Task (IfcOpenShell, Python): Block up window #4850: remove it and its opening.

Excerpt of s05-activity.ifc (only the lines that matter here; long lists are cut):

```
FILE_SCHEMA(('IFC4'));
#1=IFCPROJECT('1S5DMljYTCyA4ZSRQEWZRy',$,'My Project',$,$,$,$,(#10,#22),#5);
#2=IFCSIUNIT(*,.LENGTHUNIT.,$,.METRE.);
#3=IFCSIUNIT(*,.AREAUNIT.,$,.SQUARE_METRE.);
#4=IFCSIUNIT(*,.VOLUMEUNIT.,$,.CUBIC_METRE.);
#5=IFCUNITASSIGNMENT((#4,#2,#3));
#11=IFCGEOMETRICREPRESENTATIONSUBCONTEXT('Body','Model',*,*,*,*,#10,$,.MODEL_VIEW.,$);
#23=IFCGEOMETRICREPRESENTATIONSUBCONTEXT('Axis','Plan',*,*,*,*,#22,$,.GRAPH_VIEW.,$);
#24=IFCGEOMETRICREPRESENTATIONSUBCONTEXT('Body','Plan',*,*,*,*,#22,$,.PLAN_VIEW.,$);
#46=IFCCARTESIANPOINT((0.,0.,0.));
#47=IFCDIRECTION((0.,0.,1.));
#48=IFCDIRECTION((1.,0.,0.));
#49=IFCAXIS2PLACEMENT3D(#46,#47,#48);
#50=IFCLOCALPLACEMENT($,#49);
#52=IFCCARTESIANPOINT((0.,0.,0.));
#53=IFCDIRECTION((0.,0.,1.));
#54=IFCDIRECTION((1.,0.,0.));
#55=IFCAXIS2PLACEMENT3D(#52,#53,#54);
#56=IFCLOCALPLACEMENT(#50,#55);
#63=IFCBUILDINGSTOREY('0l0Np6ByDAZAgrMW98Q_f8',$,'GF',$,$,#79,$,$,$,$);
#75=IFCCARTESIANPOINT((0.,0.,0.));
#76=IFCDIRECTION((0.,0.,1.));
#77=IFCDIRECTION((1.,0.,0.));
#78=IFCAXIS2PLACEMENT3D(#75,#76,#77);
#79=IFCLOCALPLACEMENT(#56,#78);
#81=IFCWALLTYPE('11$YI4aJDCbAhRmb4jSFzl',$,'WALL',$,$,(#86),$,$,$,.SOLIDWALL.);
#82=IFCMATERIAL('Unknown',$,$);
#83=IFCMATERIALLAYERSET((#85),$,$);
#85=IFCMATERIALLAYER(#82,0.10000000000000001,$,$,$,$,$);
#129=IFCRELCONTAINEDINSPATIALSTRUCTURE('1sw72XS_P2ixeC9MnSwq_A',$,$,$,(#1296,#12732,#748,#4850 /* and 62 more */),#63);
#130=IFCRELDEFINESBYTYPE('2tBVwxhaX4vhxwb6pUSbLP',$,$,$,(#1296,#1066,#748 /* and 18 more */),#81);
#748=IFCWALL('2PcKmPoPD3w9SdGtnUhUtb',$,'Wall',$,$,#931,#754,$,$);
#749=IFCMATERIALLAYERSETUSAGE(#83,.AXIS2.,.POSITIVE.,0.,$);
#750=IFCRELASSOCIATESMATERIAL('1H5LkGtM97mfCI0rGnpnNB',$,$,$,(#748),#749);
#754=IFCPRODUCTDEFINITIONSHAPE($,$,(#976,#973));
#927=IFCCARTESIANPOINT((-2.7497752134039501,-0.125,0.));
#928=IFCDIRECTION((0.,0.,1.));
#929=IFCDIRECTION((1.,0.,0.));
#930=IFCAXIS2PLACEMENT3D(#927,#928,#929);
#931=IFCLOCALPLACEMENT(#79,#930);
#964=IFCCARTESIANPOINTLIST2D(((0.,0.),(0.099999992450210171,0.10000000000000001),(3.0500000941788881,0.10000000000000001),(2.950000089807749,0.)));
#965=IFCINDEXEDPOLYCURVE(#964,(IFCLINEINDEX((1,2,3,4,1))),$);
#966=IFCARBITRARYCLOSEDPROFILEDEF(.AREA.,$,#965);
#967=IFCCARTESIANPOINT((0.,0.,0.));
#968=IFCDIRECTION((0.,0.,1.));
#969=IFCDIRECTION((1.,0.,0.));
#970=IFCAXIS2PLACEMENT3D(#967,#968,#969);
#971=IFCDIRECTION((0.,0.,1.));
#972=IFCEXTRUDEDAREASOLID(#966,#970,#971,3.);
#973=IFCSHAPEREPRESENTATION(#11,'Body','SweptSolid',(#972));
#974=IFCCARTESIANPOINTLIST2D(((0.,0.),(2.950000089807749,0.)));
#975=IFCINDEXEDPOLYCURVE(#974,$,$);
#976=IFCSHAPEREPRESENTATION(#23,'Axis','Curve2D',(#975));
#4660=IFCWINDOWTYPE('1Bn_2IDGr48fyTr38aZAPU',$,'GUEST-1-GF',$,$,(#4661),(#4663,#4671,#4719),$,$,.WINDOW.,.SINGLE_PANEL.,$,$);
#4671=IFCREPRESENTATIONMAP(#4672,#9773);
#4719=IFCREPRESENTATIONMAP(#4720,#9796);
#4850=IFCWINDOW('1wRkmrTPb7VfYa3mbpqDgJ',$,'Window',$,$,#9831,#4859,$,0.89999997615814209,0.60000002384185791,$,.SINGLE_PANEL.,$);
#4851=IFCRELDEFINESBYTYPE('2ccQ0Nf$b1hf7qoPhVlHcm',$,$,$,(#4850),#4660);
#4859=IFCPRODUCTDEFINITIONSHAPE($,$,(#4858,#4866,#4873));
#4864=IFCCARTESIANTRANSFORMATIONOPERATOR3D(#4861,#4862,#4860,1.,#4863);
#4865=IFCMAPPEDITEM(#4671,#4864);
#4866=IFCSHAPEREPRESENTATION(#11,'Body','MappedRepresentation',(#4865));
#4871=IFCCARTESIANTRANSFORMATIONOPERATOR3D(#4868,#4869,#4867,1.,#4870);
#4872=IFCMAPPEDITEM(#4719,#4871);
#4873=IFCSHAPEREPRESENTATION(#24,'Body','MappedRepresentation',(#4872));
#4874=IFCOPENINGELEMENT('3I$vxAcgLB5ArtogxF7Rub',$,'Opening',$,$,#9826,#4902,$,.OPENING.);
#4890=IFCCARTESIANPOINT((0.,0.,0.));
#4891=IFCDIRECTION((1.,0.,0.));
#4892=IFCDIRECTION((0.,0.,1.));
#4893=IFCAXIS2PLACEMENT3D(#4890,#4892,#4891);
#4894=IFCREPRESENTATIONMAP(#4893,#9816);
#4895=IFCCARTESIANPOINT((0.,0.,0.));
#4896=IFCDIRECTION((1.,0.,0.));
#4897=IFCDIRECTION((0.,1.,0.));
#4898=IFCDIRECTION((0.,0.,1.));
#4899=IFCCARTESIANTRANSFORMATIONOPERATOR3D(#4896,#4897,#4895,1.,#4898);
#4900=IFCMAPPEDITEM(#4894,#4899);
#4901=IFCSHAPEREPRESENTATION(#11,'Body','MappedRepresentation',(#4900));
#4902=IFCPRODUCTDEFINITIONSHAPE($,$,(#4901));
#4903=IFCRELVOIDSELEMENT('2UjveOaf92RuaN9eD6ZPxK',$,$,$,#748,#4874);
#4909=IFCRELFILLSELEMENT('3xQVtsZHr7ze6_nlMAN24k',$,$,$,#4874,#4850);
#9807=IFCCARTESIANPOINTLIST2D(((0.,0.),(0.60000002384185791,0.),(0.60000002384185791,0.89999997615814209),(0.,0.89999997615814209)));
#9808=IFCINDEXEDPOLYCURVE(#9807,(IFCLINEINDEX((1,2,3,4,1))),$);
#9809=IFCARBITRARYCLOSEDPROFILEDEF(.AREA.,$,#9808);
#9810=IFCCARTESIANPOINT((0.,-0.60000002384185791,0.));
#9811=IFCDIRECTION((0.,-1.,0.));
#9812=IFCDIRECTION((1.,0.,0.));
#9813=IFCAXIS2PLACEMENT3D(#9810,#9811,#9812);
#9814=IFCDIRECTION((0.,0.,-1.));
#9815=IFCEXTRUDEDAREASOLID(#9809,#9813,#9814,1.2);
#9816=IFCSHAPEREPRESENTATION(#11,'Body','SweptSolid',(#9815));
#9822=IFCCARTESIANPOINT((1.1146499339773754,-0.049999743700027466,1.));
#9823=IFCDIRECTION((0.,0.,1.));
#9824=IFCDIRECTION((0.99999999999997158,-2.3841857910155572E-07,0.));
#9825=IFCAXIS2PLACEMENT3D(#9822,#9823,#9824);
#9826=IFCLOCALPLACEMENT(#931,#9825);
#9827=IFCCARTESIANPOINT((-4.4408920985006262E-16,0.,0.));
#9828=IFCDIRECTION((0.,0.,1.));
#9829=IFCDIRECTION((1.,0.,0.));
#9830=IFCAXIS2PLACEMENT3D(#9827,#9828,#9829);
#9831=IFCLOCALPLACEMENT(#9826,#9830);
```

```python
import ifcopenshell
import ifcopenshell.api.feature
import ifcopenshell.api.root
import ifcopenshell.geom
import ifcopenshell.util.shape

model = ifcopenshell.open("s05-activity.ifc")
settings = ifcopenshell.geom.settings()


def volume(element):
    """Net volume in cubic metres, openings subtracted."""
    shape = ifcopenshell.geom.create_shape(settings, element)
    return ifcopenshell.util.shape.get_volume(shape.geometry)


window = model.by_guid("1wRkmrTPb7VfYa3mbpqDgJ")
opening = window.FillsVoids[0].RelatingOpeningElement
wall = opening.VoidsElements[0].RelatingBuildingElement
before = volume(wall)

ifcopenshell.api.root.remove_product(model, product=window)
ifcopenshell.api.feature.remove_feature(model, feature=opening)

after = volume(wall)

print(f"wall volume {before:.3f} -> {after:.3f} m3")

model.write("s05-activity_edited.ifc")
```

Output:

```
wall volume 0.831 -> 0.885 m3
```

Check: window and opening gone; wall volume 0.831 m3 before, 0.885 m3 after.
